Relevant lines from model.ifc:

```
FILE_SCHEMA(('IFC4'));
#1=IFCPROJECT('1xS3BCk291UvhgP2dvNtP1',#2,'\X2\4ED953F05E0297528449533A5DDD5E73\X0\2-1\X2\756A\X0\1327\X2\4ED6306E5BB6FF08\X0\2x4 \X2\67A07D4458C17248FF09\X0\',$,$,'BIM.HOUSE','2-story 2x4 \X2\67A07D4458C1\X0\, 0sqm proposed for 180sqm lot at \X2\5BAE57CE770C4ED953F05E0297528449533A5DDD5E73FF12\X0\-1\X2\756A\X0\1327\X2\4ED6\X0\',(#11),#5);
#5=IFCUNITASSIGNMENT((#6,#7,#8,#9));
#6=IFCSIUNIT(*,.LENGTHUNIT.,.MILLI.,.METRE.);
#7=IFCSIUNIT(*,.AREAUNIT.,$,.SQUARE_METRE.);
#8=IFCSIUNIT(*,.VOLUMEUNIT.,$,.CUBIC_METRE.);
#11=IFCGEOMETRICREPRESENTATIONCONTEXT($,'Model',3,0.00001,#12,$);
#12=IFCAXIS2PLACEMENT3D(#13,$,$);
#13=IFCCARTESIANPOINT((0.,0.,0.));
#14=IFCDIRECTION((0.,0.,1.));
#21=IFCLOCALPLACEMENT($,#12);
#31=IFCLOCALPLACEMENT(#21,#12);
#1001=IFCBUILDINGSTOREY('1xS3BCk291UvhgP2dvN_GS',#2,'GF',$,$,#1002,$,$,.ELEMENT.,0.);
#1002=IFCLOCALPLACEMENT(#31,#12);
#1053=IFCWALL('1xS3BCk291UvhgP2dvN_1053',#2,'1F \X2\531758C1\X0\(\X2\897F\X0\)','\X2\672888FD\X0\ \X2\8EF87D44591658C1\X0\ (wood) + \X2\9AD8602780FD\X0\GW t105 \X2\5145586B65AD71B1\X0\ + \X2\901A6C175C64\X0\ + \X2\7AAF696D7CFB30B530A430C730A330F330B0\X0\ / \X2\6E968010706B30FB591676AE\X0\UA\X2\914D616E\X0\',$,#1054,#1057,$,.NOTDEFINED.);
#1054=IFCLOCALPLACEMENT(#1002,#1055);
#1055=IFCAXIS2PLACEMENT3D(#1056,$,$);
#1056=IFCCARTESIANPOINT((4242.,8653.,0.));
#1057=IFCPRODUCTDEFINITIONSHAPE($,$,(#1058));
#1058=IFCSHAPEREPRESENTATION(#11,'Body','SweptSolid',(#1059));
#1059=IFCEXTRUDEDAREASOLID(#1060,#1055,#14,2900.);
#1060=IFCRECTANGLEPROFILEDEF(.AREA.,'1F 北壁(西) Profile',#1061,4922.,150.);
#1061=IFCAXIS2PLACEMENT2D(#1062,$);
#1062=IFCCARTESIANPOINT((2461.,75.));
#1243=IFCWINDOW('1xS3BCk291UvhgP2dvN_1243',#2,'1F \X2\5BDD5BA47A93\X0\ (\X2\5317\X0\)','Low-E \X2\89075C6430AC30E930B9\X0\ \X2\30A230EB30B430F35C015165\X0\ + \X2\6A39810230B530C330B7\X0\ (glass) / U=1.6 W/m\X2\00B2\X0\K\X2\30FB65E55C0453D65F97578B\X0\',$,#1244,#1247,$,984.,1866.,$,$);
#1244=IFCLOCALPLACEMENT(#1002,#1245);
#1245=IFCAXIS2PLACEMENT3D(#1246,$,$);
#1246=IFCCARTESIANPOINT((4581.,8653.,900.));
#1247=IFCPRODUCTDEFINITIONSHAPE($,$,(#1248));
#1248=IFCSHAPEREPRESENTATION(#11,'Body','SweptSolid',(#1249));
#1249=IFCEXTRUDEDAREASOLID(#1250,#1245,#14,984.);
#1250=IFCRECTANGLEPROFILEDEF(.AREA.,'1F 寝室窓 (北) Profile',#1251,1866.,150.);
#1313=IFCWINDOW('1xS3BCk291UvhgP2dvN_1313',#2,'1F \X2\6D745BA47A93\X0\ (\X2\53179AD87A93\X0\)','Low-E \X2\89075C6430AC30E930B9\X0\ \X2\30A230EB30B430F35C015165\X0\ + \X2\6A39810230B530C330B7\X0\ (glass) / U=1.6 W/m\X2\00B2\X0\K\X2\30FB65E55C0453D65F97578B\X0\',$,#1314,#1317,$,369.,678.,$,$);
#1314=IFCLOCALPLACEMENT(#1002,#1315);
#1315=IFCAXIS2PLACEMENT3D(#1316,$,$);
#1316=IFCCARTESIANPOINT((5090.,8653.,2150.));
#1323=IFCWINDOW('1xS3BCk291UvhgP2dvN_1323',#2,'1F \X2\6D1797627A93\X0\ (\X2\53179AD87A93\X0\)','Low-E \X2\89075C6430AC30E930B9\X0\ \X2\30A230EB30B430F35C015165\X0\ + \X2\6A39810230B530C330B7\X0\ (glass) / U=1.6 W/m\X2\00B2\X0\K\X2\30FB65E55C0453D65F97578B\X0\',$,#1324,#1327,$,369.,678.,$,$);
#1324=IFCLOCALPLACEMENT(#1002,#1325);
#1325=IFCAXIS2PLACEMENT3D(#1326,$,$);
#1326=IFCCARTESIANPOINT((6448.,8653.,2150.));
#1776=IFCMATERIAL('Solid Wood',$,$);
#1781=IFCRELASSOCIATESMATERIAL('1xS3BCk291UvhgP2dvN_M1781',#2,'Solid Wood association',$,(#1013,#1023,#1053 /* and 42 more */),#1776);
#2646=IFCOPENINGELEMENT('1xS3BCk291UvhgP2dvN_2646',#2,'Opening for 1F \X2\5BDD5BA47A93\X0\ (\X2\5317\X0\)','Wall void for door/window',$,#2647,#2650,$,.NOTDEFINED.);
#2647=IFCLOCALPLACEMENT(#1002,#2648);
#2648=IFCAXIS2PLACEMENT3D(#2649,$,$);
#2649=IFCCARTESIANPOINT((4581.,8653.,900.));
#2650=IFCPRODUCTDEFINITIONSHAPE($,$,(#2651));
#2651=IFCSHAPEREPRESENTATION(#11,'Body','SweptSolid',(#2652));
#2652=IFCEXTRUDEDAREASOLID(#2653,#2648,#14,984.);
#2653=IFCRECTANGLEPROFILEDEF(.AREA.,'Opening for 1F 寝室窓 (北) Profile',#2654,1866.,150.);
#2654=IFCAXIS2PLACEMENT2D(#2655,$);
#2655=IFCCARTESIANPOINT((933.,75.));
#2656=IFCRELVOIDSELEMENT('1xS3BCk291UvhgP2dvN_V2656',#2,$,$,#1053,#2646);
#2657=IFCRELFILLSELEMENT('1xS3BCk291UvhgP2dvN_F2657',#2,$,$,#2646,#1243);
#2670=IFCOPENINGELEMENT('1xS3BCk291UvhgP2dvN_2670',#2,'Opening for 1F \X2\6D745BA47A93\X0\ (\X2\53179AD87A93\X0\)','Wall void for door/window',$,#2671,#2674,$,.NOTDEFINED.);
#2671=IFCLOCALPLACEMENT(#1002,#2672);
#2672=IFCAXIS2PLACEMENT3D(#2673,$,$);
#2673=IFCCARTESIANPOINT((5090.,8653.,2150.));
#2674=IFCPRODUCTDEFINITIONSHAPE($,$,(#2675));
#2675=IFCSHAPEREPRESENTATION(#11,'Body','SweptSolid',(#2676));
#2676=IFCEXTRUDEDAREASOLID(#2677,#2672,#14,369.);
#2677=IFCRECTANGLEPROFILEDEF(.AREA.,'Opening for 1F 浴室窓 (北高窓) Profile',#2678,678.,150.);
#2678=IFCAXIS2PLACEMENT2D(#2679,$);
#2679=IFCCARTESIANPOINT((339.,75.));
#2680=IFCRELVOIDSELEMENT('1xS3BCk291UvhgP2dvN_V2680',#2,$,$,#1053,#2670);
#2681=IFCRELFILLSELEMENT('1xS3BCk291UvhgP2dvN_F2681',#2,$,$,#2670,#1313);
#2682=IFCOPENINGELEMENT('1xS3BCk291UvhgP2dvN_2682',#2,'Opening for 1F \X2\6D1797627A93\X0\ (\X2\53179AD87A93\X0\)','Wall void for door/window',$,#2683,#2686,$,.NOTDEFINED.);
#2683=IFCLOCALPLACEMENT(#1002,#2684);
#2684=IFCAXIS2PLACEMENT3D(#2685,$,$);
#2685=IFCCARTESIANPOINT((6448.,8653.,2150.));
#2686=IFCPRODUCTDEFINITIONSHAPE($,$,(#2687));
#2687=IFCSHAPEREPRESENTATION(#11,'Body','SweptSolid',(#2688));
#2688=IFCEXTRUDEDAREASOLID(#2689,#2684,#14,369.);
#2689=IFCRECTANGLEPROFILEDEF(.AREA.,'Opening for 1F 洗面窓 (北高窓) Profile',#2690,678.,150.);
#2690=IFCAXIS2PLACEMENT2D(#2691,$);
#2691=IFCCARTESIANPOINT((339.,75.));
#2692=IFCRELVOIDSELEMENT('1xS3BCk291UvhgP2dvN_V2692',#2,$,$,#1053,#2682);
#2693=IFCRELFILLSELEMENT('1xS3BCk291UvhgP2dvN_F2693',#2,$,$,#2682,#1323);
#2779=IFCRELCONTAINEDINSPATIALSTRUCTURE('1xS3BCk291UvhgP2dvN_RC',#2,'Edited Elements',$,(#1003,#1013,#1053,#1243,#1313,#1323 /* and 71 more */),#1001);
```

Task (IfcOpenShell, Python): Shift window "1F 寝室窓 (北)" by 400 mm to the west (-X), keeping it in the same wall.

```python
import ifcopenshell
import ifcopenshell.api.geometry
import ifcopenshell.util.placement
import ifcopenshell.util.unit

model = ifcopenshell.open("model.ifc")
unit_scale = ifcopenshell.util.unit.calculate_unit_scale(model)

window = model.by_guid("1xS3BCk291UvhgP2dvN_1243")
opening = window.FillsVoids[0].RelatingOpeningElement
wall = opening.VoidsElements[0].RelatingBuildingElement

wall_matrix = ifcopenshell.util.placement.get_local_placement(wall.ObjectPlacement)
shift = wall_matrix[:3, 0] * -0.4 / unit_scale
before = ifcopenshell.util.placement.get_local_placement(window.ObjectPlacement)[:3, 3].copy()

# The window is not placed relative to its opening, so move both.
for product in (opening, window):
    matrix = ifcopenshell.util.placement.get_local_placement(product.ObjectPlacement)
    matrix[:3, 3] += shift
    ifcopenshell.api.geometry.edit_object_placement(model, product=product, matrix=matrix, is_si=False)

after = ifcopenshell.util.placement.get_local_placement(window.ObjectPlacement)[:3, 3]
print("window moved by", (after - before).round(3) + 0.0)

model.write("model_v2.ifc")
```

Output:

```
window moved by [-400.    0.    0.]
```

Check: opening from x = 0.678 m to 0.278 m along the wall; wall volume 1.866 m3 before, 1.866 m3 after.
